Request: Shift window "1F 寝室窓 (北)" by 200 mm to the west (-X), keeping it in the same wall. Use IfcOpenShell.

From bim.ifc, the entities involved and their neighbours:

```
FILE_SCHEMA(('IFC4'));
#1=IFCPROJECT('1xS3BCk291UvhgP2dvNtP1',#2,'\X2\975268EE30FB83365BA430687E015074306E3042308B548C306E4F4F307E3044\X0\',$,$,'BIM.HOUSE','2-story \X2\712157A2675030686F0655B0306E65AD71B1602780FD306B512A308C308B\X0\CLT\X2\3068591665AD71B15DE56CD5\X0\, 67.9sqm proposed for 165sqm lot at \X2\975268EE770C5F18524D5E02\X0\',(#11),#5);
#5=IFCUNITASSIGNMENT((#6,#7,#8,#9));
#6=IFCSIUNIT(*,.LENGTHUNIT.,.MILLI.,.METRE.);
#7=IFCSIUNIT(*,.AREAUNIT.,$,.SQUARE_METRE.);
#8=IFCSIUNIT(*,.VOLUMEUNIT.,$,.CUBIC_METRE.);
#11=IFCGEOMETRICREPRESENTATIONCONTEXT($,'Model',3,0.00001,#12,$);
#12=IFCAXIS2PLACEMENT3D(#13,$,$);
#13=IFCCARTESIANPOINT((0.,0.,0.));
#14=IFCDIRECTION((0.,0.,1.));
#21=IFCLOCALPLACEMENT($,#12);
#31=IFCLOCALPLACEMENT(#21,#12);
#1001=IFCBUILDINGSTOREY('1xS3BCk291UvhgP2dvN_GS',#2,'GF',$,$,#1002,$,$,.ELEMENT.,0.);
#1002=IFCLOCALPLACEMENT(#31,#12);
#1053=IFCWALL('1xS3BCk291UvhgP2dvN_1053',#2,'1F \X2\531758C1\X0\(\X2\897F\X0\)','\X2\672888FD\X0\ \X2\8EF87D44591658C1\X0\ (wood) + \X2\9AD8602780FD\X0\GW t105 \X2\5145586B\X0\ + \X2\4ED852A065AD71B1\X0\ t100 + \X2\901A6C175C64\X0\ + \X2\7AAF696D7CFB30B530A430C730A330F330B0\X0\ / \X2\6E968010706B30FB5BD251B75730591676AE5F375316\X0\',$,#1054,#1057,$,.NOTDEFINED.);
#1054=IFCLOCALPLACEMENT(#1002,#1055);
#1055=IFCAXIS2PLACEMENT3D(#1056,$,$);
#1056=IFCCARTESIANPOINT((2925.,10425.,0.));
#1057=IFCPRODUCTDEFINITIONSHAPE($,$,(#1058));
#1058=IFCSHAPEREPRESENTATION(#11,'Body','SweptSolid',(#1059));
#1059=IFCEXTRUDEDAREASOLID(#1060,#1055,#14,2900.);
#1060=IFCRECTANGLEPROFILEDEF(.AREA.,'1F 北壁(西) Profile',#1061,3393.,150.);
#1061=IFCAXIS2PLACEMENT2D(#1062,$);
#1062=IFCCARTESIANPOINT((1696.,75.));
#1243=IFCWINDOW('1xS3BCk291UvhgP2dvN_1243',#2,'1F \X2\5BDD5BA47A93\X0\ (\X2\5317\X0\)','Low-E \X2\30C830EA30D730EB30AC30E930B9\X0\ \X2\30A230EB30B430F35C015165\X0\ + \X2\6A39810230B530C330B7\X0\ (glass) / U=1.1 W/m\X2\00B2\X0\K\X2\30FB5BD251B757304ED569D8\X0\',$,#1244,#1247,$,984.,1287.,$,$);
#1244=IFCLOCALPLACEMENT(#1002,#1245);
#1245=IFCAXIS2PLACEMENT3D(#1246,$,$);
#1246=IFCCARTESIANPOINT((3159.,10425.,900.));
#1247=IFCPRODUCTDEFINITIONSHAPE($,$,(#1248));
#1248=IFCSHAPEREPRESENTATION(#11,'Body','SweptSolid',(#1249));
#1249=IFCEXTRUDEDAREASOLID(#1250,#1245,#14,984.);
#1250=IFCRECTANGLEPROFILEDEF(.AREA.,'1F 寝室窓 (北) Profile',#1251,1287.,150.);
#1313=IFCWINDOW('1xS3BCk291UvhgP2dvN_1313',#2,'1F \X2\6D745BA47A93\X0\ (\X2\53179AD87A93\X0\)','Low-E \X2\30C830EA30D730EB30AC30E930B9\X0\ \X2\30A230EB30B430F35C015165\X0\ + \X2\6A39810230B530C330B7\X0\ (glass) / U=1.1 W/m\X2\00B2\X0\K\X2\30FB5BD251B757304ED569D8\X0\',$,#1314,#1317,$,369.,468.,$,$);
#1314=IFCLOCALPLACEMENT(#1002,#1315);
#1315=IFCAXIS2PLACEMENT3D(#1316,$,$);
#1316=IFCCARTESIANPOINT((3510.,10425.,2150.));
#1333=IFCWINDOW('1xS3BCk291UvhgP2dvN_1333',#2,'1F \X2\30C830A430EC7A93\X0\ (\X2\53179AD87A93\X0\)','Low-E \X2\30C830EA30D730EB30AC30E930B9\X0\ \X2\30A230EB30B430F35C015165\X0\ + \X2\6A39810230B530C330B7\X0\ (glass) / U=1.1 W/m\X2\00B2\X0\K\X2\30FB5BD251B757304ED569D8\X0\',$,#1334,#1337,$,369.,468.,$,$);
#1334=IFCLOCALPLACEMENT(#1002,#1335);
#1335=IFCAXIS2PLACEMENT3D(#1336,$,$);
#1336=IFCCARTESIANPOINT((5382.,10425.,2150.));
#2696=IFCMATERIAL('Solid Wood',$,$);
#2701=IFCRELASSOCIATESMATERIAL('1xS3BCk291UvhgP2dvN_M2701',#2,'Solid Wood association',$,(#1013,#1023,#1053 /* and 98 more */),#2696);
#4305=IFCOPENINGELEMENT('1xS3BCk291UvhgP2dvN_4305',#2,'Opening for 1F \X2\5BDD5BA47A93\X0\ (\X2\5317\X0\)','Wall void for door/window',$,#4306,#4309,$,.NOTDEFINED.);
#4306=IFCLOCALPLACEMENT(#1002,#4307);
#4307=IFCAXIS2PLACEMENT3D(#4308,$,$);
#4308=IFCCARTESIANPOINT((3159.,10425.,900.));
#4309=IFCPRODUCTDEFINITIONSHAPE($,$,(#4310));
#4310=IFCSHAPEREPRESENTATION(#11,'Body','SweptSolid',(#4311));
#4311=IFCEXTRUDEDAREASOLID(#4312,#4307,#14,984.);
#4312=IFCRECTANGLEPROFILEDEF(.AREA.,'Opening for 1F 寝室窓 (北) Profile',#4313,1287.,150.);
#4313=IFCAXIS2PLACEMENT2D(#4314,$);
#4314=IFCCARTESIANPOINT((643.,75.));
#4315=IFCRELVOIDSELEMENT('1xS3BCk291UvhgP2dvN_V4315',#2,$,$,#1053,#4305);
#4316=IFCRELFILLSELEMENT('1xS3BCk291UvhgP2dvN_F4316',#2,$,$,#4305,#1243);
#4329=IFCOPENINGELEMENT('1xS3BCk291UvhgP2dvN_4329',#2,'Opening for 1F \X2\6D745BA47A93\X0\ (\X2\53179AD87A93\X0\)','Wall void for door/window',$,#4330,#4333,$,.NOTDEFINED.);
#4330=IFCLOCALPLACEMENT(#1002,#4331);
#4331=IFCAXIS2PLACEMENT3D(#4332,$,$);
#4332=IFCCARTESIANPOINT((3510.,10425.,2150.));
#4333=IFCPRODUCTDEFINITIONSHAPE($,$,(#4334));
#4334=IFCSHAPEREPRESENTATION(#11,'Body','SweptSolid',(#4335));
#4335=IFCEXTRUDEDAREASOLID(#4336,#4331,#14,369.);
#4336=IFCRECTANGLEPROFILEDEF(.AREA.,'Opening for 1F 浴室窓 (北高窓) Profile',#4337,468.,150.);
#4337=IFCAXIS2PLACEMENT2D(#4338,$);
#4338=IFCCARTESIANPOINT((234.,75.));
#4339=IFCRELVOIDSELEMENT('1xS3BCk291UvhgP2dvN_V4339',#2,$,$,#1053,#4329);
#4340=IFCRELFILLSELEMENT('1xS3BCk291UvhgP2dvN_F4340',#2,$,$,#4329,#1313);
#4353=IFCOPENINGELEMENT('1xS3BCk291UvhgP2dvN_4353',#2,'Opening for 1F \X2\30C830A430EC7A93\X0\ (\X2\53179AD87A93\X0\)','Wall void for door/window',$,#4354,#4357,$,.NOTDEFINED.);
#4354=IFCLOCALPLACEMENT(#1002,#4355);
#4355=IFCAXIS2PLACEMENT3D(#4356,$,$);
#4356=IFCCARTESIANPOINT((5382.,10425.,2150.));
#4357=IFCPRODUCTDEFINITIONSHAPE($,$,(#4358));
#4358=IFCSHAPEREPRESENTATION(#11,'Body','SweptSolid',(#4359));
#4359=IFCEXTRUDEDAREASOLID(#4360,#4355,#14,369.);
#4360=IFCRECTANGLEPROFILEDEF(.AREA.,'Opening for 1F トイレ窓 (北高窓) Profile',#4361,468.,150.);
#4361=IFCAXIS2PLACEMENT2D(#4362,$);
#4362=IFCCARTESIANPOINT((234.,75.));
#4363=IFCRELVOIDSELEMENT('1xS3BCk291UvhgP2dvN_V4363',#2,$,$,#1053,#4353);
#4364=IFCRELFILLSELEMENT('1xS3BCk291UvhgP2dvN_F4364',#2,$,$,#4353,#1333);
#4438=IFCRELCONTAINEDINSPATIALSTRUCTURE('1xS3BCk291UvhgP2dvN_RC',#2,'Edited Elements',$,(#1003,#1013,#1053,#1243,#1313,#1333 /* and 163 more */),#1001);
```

```python
import ifcopenshell
import ifcopenshell.api.geometry
import ifcopenshell.util.placement

model = ifcopenshell.open("bim.ifc")

window = model.by_guid("1xS3BCk291UvhgP2dvN_1243")
opening = window.FillsVoids[0].RelatingOpeningElement
wall = opening.VoidsElements[0].RelatingBuildingElement

wall_matrix = ifcopenshell.util.placement.get_local_placement(wall.ObjectPlacement)
shift = wall_matrix[:3, 0] * -200.0
before = ifcopenshell.util.placement.get_local_placement(window.ObjectPlacement)[:3, 3].copy()

# The window is not placed relative to its opening, so move both.
for product in (opening, window):
    matrix = ifcopenshell.util.placement.get_local_placement(product.ObjectPlacement)
    matrix[:3, 3] += shift
    ifcopenshell.api.geometry.edit_object_placement(model, product=product, matrix=matrix, is_si=False)

after = ifcopenshell.util.placement.get_local_placement(window.ObjectPlacement)[:3, 3]
print("window moved by", (after - before).round(3) + 0.0)

model.write("bim_edited.ifc")
```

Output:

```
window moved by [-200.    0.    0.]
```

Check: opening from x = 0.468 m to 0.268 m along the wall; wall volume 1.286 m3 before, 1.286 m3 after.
